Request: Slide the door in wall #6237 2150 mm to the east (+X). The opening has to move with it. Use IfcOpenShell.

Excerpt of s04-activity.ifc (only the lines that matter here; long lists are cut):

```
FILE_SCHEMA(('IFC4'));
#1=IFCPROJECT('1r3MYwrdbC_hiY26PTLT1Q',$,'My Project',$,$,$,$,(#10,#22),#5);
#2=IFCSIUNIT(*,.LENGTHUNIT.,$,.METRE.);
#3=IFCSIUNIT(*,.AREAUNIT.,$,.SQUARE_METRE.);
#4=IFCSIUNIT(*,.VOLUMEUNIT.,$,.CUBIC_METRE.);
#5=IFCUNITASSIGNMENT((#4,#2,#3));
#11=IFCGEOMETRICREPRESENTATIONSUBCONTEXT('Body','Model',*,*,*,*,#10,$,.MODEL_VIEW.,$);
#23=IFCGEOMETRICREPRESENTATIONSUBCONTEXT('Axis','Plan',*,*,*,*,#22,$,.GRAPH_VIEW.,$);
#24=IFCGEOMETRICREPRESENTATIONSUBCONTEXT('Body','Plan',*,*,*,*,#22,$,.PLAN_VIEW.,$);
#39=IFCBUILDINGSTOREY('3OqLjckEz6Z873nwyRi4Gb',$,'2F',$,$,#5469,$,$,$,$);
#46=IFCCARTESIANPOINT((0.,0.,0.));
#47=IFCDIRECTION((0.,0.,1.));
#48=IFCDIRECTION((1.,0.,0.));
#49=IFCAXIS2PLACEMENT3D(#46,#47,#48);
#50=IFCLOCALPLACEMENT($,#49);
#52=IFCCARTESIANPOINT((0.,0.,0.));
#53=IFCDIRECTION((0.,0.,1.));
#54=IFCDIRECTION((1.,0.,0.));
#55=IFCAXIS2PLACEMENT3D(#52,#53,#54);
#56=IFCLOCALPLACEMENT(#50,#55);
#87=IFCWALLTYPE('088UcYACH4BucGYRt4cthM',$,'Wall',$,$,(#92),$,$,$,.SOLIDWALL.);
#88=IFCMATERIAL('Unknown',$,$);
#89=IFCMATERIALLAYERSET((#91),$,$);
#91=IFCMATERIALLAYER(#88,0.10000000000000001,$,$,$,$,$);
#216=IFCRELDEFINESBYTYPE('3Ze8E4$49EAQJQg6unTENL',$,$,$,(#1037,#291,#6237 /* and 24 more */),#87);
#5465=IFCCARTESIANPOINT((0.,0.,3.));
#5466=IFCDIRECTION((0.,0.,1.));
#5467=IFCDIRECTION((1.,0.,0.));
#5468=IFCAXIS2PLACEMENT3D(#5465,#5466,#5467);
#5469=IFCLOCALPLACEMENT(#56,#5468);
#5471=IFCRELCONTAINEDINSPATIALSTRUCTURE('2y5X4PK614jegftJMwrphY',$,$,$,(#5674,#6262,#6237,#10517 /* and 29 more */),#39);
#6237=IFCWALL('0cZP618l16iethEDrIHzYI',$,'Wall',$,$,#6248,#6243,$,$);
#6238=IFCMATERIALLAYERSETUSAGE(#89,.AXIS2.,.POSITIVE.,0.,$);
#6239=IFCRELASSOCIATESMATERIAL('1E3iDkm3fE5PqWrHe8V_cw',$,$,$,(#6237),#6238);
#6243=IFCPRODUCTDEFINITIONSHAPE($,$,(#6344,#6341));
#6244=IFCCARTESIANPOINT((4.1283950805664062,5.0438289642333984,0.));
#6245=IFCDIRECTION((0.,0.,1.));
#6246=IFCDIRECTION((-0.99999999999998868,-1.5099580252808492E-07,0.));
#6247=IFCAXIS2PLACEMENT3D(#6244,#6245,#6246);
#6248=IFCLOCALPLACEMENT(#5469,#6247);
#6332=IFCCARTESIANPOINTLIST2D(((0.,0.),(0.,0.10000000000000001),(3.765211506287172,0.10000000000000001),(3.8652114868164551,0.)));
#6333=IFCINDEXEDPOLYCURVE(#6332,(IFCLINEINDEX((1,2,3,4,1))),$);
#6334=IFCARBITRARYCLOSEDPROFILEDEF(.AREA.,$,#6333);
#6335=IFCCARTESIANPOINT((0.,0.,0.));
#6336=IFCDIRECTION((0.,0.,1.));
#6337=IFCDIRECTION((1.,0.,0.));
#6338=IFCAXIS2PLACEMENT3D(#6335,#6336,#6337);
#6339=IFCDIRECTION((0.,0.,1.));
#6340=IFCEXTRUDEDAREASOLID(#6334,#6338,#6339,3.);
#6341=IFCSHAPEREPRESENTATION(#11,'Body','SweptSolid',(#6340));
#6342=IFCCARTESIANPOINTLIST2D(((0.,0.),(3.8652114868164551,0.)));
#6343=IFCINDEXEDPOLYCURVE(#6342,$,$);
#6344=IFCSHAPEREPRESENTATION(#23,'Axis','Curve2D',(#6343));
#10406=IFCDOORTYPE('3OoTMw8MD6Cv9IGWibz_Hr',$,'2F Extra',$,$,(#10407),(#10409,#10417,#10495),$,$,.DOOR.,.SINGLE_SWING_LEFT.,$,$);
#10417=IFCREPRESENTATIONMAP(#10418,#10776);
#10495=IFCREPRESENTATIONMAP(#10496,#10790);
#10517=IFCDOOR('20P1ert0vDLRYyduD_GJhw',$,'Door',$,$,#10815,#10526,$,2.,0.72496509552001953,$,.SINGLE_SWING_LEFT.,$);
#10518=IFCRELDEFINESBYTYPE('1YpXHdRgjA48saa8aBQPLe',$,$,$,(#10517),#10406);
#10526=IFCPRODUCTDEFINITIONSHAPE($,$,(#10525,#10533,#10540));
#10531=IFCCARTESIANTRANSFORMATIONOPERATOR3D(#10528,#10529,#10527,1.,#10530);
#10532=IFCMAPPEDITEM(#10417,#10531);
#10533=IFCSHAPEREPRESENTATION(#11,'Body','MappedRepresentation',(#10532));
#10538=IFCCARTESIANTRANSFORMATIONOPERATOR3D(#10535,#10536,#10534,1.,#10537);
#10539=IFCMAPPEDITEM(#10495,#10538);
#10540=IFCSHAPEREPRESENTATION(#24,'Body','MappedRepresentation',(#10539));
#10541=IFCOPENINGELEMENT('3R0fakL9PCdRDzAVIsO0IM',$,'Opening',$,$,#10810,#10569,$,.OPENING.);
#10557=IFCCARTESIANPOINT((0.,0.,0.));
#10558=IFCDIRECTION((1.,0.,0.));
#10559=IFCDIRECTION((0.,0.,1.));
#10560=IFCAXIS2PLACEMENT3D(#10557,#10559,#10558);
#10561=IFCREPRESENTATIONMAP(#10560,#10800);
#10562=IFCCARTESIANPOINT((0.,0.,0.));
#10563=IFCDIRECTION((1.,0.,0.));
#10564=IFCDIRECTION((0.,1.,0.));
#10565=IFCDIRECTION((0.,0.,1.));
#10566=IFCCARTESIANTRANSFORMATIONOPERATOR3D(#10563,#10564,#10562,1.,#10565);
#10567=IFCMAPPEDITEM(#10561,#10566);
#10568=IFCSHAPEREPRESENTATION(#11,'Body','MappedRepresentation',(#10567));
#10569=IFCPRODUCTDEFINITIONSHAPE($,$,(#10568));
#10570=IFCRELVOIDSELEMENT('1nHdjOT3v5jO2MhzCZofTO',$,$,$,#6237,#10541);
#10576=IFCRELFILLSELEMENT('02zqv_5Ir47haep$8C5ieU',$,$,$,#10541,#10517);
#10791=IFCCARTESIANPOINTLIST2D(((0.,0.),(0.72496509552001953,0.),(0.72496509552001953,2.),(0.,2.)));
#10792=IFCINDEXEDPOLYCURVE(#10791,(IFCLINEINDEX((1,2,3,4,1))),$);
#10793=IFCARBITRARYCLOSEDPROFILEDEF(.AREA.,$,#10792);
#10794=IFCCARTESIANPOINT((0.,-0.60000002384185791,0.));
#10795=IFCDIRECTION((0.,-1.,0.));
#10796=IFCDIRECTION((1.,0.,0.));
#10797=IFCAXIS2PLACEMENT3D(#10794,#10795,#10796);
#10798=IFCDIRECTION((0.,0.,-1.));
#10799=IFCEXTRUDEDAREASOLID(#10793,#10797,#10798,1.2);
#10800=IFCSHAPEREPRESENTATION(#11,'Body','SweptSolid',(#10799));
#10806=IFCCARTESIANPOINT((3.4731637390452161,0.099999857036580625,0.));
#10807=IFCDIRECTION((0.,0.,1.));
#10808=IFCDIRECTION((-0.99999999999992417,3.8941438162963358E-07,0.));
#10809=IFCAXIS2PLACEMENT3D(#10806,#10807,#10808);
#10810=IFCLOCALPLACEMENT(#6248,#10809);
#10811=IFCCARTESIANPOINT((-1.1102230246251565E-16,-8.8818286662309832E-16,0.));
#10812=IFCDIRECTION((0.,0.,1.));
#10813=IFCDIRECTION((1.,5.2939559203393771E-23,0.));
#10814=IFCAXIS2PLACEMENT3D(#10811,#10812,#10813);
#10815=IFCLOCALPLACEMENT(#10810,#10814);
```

```python
import ifcopenshell
import ifcopenshell.api.geometry
import ifcopenshell.util.placement

model = ifcopenshell.open("s04-activity.ifc")

door = model.by_guid("20P1ert0vDLRYyduD_GJhw")
opening = door.FillsVoids[0].RelatingOpeningElement
wall = opening.VoidsElements[0].RelatingBuildingElement

wall_matrix = ifcopenshell.util.placement.get_local_placement(wall.ObjectPlacement)
shift = wall_matrix[:3, 0] * -2.15
before = ifcopenshell.util.placement.get_local_placement(door.ObjectPlacement)[:3, 3].copy()

# The door is placed relative to its opening, so it follows when the opening moves.
matrix = ifcopenshell.util.placement.get_local_placement(opening.ObjectPlacement)
matrix[:3, 3] += shift
ifcopenshell.api.geometry.edit_object_placement(
    model, product=opening, matrix=matrix, is_si=False, should_transform_children=True
)

after = ifcopenshell.util.placement.get_local_placement(door.ObjectPlacement)[:3, 3]
print("door moved by", (after - before).round(3) + 0.0)

model.write("s04-activity_v2.ifc")
```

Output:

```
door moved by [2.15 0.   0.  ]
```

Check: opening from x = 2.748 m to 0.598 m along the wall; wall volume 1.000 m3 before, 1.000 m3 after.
